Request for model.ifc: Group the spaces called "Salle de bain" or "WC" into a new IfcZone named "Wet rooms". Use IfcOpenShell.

First a look at what the model holds.

```python
import ifcopenshell

model = ifcopenshell.open("model.ifc")
print(model.schema)
seen = {}
for space in model.by_type("IfcSpace"):
    seen[space.LongName] = seen.get(space.LongName, 0) + 1
for name, count in sorted(seen.items(), key=str):
    print(count, "x", name)
print("zones:", [z.Name for z in model.by_type("IfcZone")][:20])
```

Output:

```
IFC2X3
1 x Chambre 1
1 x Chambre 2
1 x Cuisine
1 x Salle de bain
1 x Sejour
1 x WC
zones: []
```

```python
import ifcopenshell
import ifcopenshell.api.group
import ifcopenshell.api.root

model = ifcopenshell.open("model.ifc")

names = {"Salle de bain", "WC"}
spaces = [s for s in model.by_type("IfcSpace") if s.LongName in names]

zone = ifcopenshell.api.root.create_entity(model, ifc_class="IfcZone", name="Wet rooms")
ifcopenshell.api.group.assign_group(model, products=spaces, group=zone)
print(len(spaces), "spaces in", zone.Name)

model.write("model_v2.ifc")
```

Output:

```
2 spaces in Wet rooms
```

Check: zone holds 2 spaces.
